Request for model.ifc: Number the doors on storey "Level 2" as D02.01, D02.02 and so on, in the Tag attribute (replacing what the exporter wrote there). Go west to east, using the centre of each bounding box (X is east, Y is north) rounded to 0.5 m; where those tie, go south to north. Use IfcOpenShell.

First a look at what the model holds.

```python
import ifcopenshell
import ifcopenshell.util.element
import ifcopenshell.util.placement

model = ifcopenshell.open("model.ifc")
print(model.schema)
storey = next(s for s in model.by_type("IfcBuildingStorey") if s.Name == "Level 2")
doors = [e for e in ifcopenshell.util.element.get_decomposition(storey) if e.is_a("IfcDoor")]
for e in sorted(doors, key=lambda e: e.id()):
    origin = ifcopenshell.util.placement.get_local_placement(e.ObjectPlacement)[:3, 3]
    print(e.id(), e.Tag, e.Name, origin.round(2) + 0.0, sep=" | ")
```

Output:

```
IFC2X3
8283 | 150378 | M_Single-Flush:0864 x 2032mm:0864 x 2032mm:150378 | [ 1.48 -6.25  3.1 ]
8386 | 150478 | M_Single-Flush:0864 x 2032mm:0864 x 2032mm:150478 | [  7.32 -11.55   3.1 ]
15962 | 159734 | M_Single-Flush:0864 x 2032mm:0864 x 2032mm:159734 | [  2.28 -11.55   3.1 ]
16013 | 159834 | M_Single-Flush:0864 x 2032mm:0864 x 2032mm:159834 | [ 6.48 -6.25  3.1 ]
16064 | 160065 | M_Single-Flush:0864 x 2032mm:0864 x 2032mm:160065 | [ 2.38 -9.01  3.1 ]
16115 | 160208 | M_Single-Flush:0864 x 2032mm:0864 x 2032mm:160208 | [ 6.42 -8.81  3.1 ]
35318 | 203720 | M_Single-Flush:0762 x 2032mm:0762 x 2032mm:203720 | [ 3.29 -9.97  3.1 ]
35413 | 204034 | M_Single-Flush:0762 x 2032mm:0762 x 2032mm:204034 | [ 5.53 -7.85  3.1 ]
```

```python
import ifcopenshell
import ifcopenshell.geom
import ifcopenshell.util.element
import ifcopenshell.util.shape

model = ifcopenshell.open("model.ifc")
settings = ifcopenshell.geom.settings()
settings.set("use-world-coords", True)


def centre(element):
    shape = ifcopenshell.geom.create_shape(settings, element)
    return ifcopenshell.util.shape.get_bbox_centroid(shape.geometry)


storey = next(s for s in model.by_type("IfcBuildingStorey") if s.Name == "Level 2")
doors = [e for e in ifcopenshell.util.element.get_decomposition(storey) if e.is_a("IfcDoor")]

# Insertion points can sit at a corner or the storey origin, so sort by the geometry (in metres).
centres = {e: centre(e) for e in doors}
doors.sort(key=lambda e: (round(centres[e][0] / 0.5), centres[e][1]))

for i, e in enumerate(doors, start=1):
    number = f"D02.{i:02d}"
    e.Tag = number
    print(e.id(), number)

model.write("model_v2.ifc")
```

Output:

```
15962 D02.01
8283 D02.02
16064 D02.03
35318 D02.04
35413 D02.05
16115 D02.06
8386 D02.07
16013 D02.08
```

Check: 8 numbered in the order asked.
